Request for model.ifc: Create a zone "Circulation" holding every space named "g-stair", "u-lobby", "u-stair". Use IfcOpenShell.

First a look at what the model holds.

```python
import ifcopenshell

model = ifcopenshell.open("model.ifc")
print(model.schema)
seen = {}
for space in model.by_type("IfcSpace"):
    seen[space.LongName] = seen.get(space.LongName, 0) + 1
for name, count in sorted(seen.items(), key=str):
    print(count, "x", name)
print("zones:", [z.Name for z in model.by_type("IfcZone")][:20])
```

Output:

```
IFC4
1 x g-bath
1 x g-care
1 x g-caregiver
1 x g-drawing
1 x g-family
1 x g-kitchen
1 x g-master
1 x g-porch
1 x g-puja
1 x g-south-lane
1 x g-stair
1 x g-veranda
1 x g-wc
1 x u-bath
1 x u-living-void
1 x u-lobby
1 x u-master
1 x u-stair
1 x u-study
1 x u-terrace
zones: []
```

```python
import ifcopenshell
import ifcopenshell.api.group
import ifcopenshell.api.root

model = ifcopenshell.open("model.ifc")

names = {"g-stair", "u-lobby", "u-stair"}
spaces = [s for s in model.by_type("IfcSpace") if s.LongName in names]

zone = ifcopenshell.api.root.create_entity(model, ifc_class="IfcZone", name="Circulation")
ifcopenshell.api.group.assign_group(model, products=spaces, group=zone)
print(len(spaces), "spaces in", zone.Name)

model.write("model_rev.ifc")
```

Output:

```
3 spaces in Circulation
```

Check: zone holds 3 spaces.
